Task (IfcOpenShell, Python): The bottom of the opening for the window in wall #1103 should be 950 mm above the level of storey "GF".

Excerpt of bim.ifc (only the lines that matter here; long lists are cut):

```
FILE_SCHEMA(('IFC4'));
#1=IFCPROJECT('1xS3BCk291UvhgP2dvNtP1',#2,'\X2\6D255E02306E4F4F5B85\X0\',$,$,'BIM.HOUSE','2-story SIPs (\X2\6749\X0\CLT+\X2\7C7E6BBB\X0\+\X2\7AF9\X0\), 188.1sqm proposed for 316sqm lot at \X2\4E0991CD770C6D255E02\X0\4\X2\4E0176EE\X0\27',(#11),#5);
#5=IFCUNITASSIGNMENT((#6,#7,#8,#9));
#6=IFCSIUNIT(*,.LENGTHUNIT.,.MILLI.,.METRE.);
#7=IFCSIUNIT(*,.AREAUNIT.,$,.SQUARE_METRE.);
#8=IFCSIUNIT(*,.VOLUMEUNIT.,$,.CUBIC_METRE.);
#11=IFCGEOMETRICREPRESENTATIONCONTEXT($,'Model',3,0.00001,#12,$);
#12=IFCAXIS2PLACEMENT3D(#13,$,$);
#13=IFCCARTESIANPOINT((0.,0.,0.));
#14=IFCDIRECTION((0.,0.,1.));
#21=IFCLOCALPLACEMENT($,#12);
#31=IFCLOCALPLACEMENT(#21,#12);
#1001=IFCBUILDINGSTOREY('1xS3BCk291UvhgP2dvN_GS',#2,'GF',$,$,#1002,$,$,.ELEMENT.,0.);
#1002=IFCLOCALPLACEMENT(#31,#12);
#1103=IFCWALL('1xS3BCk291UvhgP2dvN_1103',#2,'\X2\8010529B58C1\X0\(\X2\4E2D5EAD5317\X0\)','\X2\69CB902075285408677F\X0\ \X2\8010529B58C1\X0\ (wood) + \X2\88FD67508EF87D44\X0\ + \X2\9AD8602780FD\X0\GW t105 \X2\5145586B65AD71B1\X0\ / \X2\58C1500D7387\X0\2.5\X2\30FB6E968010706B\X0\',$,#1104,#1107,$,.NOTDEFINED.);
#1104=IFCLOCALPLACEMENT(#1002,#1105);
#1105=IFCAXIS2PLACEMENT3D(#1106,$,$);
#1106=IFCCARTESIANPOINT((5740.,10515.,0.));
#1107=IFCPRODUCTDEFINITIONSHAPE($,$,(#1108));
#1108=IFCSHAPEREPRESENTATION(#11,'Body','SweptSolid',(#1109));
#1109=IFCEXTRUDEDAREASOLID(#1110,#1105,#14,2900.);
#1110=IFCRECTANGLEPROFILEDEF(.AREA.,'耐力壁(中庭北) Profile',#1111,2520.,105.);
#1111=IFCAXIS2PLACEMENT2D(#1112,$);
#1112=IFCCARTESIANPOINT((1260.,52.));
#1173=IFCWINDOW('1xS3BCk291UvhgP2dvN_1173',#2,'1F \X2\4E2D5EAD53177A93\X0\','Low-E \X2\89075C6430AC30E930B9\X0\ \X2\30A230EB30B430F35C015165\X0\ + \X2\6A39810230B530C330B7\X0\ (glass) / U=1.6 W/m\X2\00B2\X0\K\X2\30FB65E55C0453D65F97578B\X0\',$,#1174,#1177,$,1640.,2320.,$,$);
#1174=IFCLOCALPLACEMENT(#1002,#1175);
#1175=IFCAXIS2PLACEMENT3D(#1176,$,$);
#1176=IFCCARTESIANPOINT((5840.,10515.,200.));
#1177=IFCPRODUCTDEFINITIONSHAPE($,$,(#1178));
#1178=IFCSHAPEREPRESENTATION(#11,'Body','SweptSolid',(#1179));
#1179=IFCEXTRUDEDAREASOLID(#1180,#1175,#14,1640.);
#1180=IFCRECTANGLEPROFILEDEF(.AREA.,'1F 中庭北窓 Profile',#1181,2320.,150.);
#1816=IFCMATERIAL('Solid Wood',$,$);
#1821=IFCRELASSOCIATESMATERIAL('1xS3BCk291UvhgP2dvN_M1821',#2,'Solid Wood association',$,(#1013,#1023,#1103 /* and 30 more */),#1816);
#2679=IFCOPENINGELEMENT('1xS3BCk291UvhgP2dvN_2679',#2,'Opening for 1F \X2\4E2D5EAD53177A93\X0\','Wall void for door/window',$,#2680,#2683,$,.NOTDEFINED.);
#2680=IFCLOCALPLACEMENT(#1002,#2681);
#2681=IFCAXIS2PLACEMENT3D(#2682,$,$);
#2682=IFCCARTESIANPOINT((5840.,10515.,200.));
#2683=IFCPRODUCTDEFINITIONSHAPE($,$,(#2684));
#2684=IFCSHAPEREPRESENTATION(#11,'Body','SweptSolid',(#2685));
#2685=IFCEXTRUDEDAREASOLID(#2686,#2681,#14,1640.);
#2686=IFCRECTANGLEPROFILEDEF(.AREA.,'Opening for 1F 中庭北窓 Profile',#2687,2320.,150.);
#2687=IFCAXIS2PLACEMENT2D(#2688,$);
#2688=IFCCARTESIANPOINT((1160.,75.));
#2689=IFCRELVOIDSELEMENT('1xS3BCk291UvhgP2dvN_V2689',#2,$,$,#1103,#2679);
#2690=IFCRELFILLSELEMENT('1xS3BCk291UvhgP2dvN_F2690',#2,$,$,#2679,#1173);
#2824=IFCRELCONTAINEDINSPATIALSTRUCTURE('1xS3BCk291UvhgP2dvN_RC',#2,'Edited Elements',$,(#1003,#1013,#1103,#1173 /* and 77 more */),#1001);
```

```python
import numpy as np
import ifcopenshell
import ifcopenshell.api.geometry
import ifcopenshell.geom
import ifcopenshell.util.element
import ifcopenshell.util.placement
import ifcopenshell.util.shape
import ifcopenshell.util.unit

model = ifcopenshell.open("bim.ifc")
unit_scale = ifcopenshell.util.unit.calculate_unit_scale(model)

window = model.by_id(1173)
opening = window.FillsVoids[0].RelatingOpeningElement
storey = ifcopenshell.util.element.get_container(window, ifc_class="IfcBuildingStorey")
level = ifcopenshell.util.placement.get_local_placement(storey.ObjectPlacement)[2, 3]

# The opening's origin need not be at the sill, so measure its lowest point.
shape = ifcopenshell.geom.create_shape(ifcopenshell.geom.settings(), opening)
bottom = ifcopenshell.util.shape.get_shape_bottom_elevation(shape, shape.geometry) / unit_scale
dz = level + 0.95 / unit_scale - bottom

shift = np.array([0.0, 0.0, dz])
# The window is not placed relative to its opening, so move both.
for product in (opening, window):
    matrix = ifcopenshell.util.placement.get_local_placement(product.ObjectPlacement)
    matrix[:3, 3] += shift
    ifcopenshell.api.geometry.edit_object_placement(model, product=product, matrix=matrix, is_si=False)

print(f"moved by {dz * unit_scale:+.3f} m")

model.write("bim_v2.ifc")
```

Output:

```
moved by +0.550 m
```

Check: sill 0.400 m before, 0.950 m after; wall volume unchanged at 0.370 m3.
